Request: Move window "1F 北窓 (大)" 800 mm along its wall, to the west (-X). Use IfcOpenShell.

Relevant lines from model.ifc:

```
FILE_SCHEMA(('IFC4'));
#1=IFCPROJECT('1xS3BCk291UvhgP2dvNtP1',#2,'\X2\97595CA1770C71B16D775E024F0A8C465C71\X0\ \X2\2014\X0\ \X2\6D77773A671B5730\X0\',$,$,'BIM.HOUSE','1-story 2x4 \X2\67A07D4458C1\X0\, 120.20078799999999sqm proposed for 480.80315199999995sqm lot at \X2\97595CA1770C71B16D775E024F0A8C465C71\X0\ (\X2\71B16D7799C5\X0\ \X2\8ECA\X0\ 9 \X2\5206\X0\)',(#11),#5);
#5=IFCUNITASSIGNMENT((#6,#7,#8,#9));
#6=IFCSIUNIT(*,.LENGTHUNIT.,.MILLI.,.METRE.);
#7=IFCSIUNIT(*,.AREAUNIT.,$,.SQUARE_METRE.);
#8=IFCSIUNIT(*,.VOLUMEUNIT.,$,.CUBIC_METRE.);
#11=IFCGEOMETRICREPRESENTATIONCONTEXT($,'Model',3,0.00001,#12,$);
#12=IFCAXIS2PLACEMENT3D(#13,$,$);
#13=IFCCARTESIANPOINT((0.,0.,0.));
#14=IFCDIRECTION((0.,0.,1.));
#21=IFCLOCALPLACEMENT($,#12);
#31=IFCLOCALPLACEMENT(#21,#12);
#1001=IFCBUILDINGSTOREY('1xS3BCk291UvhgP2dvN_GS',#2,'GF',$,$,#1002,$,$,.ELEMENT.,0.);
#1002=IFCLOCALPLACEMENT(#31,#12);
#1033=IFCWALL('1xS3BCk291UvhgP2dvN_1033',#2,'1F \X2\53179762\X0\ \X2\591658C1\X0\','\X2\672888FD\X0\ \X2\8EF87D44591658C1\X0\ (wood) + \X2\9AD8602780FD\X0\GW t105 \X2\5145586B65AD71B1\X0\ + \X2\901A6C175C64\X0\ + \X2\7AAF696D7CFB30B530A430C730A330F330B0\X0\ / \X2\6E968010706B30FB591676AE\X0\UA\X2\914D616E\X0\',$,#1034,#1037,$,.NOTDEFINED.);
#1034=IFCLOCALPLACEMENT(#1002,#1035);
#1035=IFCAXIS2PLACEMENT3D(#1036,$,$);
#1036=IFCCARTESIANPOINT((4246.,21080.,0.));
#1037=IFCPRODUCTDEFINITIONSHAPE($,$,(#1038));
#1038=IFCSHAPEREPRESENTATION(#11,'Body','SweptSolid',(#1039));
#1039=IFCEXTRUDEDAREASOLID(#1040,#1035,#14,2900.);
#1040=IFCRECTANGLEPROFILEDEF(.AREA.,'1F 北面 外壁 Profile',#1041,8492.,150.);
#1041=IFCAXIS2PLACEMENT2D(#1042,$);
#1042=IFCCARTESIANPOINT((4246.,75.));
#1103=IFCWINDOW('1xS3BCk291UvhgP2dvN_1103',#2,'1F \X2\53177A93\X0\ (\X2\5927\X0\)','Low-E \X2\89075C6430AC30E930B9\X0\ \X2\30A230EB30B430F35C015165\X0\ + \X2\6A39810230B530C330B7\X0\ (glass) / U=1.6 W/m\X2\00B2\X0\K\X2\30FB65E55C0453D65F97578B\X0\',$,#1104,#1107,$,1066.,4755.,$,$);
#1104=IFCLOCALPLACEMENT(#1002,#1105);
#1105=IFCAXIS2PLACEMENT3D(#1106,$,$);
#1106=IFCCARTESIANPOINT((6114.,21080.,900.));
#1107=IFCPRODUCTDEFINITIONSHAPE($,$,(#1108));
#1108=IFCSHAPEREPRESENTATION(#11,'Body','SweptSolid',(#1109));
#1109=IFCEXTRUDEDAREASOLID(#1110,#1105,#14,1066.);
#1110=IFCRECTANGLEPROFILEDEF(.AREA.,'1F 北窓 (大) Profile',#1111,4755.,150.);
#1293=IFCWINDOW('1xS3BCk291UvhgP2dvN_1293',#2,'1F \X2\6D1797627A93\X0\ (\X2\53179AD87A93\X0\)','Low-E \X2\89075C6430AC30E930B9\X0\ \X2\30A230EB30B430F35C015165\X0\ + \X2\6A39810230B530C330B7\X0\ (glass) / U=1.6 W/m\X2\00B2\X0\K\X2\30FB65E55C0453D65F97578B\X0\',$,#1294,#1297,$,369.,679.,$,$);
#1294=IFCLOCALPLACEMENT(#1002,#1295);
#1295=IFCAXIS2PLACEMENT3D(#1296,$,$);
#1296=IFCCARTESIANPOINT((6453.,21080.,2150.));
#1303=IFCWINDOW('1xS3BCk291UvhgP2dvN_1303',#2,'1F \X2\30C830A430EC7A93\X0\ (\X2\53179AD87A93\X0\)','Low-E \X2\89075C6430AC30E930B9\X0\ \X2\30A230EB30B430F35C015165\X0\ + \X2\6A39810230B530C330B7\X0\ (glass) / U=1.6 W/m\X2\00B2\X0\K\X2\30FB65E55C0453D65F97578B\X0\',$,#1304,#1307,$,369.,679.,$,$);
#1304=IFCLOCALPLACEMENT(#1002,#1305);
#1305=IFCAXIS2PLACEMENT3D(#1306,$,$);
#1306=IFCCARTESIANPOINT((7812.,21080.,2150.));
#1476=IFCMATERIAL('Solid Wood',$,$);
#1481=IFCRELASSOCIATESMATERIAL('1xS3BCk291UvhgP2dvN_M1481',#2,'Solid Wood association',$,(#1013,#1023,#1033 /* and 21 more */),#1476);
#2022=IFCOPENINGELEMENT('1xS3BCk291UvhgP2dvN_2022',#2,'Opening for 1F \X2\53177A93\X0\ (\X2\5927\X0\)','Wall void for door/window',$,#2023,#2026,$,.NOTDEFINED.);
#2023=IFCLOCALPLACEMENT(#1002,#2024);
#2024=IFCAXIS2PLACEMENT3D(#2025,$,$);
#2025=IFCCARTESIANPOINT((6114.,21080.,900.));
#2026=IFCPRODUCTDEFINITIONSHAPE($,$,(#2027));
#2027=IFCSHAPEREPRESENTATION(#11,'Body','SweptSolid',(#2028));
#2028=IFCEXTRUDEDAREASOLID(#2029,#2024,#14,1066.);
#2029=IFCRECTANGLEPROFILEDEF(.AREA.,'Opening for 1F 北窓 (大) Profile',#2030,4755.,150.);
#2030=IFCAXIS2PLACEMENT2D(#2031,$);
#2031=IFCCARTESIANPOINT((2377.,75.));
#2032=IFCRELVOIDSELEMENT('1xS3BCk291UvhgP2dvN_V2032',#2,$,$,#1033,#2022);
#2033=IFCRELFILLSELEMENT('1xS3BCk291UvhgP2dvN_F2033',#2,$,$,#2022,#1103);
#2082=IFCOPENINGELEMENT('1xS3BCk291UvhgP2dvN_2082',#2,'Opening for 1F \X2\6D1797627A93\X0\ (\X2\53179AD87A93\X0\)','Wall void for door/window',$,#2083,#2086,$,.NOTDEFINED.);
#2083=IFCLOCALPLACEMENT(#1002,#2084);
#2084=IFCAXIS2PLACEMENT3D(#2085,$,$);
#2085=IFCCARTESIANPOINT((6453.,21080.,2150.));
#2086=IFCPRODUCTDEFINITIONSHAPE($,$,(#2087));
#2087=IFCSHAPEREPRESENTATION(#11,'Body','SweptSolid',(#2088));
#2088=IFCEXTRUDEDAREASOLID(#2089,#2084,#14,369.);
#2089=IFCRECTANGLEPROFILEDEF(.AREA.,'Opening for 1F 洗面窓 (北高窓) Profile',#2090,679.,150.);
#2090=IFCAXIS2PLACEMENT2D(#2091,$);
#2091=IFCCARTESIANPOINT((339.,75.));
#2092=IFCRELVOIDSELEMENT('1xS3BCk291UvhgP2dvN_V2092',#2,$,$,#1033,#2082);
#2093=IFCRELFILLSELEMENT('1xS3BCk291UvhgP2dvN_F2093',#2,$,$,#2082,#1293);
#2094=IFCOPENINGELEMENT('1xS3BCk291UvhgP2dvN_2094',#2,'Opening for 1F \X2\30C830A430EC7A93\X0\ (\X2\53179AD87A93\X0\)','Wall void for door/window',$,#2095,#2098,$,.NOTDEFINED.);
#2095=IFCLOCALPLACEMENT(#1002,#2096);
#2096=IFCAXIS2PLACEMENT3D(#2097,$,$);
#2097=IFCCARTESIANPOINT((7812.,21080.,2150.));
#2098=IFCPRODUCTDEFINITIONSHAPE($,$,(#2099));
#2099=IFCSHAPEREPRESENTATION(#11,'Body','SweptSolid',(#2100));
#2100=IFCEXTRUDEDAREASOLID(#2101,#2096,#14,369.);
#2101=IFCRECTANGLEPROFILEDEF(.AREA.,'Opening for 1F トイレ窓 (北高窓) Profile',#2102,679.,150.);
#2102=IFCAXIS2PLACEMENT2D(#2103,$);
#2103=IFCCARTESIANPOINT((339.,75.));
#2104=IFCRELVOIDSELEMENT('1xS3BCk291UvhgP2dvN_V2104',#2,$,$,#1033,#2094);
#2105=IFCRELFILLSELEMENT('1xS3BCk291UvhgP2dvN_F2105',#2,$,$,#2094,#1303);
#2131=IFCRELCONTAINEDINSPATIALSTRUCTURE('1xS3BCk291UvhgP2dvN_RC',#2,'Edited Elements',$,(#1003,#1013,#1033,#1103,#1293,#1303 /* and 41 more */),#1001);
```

```python
import ifcopenshell
import ifcopenshell.api.geometry
import ifcopenshell.util.placement
import ifcopenshell.util.unit

model = ifcopenshell.open("model.ifc")
unit_scale = ifcopenshell.util.unit.calculate_unit_scale(model)

window = model.by_id(1103)
opening = window.FillsVoids[0].RelatingOpeningElement
wall = opening.VoidsElements[0].RelatingBuildingElement

wall_matrix = ifcopenshell.util.placement.get_local_placement(wall.ObjectPlacement)
shift = wall_matrix[:3, 0] * -0.8 / unit_scale
before = ifcopenshell.util.placement.get_local_placement(window.ObjectPlacement)[:3, 3].copy()

# The window is not placed relative to its opening, so move both.
for product in (opening, window):
    matrix = ifcopenshell.util.placement.get_local_placement(product.ObjectPlacement)
    matrix[:3, 3] += shift
    ifcopenshell.api.geometry.edit_object_placement(model, product=product, matrix=matrix, is_si=False)

after = ifcopenshell.util.placement.get_local_placement(window.ObjectPlacement)[:3, 3]
print("window moved by", (after - before).round(3) + 0.0)

model.write("model_updated.ifc")
```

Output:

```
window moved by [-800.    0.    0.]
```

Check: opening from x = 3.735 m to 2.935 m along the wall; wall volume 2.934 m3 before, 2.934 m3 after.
